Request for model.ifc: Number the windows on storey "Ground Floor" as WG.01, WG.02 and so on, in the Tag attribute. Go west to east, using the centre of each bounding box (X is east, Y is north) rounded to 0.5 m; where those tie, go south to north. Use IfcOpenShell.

First a look at what the model holds.

```python
import ifcopenshell
import ifcopenshell.util.element
import ifcopenshell.util.placement

model = ifcopenshell.open("model.ifc")
print(model.schema)
storey = next(s for s in model.by_type("IfcBuildingStorey") if s.Name == "Ground Floor")
windows = [e for e in ifcopenshell.util.element.get_decomposition(storey) if e.is_a("IfcWindow")]
for e in sorted(windows, key=lambda e: e.id()):
    origin = ifcopenshell.util.placement.get_local_placement(e.ObjectPlacement)[:3, 3]
    print(e.id(), e.Tag, e.Name, origin.round(2) + 0.0, sep=" | ")
```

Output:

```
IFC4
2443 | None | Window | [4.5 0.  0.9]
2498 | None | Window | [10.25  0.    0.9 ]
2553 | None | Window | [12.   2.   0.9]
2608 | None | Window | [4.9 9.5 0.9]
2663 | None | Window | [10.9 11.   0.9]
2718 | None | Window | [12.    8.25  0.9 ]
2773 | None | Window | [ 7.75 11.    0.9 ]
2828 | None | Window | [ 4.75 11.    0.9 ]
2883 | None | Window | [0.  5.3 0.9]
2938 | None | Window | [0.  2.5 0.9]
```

```python
import ifcopenshell
import ifcopenshell.geom
import ifcopenshell.util.element
import ifcopenshell.util.shape

model = ifcopenshell.open("model.ifc")
settings = ifcopenshell.geom.settings()
settings.set("use-world-coords", True)


def centre(element):
    shape = ifcopenshell.geom.create_shape(settings, element)
    return ifcopenshell.util.shape.get_bbox_centroid(shape.geometry)


storey = next(s for s in model.by_type("IfcBuildingStorey") if s.Name == "Ground Floor")
windows = [e for e in ifcopenshell.util.element.get_decomposition(storey) if e.is_a("IfcWindow")]

# Insertion points can sit at a corner or the storey origin, so sort by the geometry (in metres).
centres = {e: centre(e) for e in windows}
windows.sort(key=lambda e: (round(centres[e][0] / 0.5), centres[e][1]))

for i, e in enumerate(windows, start=1):
    number = f"WG.{i:02d}"
    e.Tag = number
    print(e.id(), number)

model.write("model-out.ifc")
```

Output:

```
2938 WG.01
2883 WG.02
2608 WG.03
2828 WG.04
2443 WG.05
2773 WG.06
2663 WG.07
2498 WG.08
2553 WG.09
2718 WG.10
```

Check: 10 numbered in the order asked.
